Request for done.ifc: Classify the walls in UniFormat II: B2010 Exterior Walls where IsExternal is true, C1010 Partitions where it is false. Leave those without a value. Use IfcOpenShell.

First a look at what the model holds.

```python
import ifcopenshell
import ifcopenshell.util.element

model = ifcopenshell.open("done.ifc")
print(model.schema)
print("classifications:", [c.Name for c in model.by_type("IfcClassification")])
values = [ifcopenshell.util.element.get_pset(e, "Pset_WallCommon", "IsExternal") for e in model.by_type("IfcWall")]
for value in (True, False, None):
    print("IsExternal", value, values.count(value))
```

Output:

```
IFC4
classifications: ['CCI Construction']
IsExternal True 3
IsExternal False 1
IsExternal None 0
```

```python
import ifcopenshell
import ifcopenshell.api.classification
import ifcopenshell.util.element

model = ifcopenshell.open("done.ifc")

system = ifcopenshell.api.classification.add_classification(model, classification="UniFormat II")

walls = model.by_type("IfcWall")
external = {e: ifcopenshell.util.element.get_pset(e, "Pset_WallCommon", "IsExternal") for e in walls}
for flag, code, name in ((True, "B2010", "Exterior Walls"), (False, "C1010", "Partitions")):
    products = [e for e in walls if external[e] is flag]
    ifcopenshell.api.classification.add_reference(
        model, products=products, classification=system, identification=code, name=name
    )
    print(code, len(products))

model.write("done_edited.ifc")
```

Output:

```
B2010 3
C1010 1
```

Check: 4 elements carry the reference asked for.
